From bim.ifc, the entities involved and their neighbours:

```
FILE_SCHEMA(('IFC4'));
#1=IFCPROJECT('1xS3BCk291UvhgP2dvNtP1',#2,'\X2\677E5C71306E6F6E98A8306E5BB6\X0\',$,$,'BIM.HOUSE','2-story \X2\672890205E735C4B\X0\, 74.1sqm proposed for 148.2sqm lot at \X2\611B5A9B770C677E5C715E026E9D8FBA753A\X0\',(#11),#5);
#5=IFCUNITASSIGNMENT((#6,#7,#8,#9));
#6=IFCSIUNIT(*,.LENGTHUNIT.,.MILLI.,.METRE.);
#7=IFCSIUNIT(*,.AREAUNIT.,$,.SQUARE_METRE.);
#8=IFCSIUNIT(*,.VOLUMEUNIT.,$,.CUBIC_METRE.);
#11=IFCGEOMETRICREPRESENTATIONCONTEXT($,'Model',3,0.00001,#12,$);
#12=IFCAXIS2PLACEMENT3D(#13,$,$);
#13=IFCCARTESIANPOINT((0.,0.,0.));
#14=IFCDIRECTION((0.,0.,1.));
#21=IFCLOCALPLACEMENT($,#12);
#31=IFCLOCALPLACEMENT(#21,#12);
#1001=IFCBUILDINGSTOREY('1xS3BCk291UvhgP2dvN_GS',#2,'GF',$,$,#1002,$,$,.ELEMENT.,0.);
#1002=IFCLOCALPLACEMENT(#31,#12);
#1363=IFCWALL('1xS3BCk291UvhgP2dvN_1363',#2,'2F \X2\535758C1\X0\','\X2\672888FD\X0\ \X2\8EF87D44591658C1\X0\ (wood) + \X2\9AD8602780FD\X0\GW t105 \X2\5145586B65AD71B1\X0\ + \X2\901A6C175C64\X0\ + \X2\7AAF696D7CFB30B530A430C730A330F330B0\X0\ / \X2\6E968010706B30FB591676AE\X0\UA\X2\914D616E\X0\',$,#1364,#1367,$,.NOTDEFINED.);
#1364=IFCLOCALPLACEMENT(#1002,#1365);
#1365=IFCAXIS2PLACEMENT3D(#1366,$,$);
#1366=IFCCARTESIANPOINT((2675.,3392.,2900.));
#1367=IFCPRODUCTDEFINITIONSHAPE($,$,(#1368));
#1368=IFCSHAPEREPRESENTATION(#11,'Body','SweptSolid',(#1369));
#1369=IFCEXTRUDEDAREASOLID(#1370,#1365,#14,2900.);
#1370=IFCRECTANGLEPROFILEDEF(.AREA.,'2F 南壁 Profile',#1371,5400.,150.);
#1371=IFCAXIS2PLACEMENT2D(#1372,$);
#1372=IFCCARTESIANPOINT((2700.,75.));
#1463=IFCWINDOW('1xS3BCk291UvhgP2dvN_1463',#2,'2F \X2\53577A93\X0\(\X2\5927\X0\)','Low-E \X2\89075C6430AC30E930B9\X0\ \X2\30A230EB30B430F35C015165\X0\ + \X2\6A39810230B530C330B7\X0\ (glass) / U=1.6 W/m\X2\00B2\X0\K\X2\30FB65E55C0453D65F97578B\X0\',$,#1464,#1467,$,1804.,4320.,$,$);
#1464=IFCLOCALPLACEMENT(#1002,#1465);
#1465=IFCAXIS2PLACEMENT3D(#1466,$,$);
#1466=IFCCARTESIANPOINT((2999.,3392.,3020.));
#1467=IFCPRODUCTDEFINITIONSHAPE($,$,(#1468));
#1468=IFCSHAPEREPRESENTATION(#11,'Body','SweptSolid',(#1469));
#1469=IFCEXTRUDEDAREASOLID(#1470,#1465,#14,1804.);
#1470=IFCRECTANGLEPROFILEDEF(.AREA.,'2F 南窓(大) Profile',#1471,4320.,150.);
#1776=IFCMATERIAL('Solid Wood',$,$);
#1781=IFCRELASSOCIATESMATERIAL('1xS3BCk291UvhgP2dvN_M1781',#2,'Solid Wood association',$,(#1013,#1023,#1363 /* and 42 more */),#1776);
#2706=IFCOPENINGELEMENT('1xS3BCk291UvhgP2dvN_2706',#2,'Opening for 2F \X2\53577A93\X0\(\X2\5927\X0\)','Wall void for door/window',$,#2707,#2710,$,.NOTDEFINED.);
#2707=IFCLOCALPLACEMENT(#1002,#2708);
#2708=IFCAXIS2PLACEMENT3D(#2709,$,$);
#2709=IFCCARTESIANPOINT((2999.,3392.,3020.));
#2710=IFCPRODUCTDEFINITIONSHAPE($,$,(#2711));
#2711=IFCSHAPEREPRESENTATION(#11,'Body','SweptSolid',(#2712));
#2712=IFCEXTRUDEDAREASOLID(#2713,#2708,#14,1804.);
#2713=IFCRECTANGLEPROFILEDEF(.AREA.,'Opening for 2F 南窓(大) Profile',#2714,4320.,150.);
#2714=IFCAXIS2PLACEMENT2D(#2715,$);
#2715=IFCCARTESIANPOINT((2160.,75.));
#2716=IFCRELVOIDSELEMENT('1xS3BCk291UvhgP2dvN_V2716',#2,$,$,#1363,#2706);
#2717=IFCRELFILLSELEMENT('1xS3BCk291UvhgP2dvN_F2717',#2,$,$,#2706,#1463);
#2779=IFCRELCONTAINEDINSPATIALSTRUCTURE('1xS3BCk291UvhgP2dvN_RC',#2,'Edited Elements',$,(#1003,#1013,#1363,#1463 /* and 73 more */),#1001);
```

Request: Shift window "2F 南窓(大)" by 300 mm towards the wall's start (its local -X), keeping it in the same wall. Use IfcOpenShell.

```python
import ifcopenshell
import ifcopenshell.api.geometry
import ifcopenshell.util.placement
import ifcopenshell.util.unit

model = ifcopenshell.open("bim.ifc")
unit_scale = ifcopenshell.util.unit.calculate_unit_scale(model)

window = model.by_guid("1xS3BCk291UvhgP2dvN_1463")
opening = window.FillsVoids[0].RelatingOpeningElement
wall = opening.VoidsElements[0].RelatingBuildingElement

wall_matrix = ifcopenshell.util.placement.get_local_placement(wall.ObjectPlacement)
shift = wall_matrix[:3, 0] * -0.3 / unit_scale
before = ifcopenshell.util.placement.get_local_placement(window.ObjectPlacement)[:3, 3].copy()

# The window is not placed relative to its opening, so move both.
for product in (opening, window):
    matrix = ifcopenshell.util.placement.get_local_placement(product.ObjectPlacement)
    matrix[:3, 3] += shift
    ifcopenshell.api.geometry.edit_object_placement(model, product=product, matrix=matrix, is_si=False)

after = ifcopenshell.util.placement.get_local_placement(window.ObjectPlacement)[:3, 3]
print("window moved by", (after - before).round(3) + 0.0)

model.write("bim_edited.ifc")
```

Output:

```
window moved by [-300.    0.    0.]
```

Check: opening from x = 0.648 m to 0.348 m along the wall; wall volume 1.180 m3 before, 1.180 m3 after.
